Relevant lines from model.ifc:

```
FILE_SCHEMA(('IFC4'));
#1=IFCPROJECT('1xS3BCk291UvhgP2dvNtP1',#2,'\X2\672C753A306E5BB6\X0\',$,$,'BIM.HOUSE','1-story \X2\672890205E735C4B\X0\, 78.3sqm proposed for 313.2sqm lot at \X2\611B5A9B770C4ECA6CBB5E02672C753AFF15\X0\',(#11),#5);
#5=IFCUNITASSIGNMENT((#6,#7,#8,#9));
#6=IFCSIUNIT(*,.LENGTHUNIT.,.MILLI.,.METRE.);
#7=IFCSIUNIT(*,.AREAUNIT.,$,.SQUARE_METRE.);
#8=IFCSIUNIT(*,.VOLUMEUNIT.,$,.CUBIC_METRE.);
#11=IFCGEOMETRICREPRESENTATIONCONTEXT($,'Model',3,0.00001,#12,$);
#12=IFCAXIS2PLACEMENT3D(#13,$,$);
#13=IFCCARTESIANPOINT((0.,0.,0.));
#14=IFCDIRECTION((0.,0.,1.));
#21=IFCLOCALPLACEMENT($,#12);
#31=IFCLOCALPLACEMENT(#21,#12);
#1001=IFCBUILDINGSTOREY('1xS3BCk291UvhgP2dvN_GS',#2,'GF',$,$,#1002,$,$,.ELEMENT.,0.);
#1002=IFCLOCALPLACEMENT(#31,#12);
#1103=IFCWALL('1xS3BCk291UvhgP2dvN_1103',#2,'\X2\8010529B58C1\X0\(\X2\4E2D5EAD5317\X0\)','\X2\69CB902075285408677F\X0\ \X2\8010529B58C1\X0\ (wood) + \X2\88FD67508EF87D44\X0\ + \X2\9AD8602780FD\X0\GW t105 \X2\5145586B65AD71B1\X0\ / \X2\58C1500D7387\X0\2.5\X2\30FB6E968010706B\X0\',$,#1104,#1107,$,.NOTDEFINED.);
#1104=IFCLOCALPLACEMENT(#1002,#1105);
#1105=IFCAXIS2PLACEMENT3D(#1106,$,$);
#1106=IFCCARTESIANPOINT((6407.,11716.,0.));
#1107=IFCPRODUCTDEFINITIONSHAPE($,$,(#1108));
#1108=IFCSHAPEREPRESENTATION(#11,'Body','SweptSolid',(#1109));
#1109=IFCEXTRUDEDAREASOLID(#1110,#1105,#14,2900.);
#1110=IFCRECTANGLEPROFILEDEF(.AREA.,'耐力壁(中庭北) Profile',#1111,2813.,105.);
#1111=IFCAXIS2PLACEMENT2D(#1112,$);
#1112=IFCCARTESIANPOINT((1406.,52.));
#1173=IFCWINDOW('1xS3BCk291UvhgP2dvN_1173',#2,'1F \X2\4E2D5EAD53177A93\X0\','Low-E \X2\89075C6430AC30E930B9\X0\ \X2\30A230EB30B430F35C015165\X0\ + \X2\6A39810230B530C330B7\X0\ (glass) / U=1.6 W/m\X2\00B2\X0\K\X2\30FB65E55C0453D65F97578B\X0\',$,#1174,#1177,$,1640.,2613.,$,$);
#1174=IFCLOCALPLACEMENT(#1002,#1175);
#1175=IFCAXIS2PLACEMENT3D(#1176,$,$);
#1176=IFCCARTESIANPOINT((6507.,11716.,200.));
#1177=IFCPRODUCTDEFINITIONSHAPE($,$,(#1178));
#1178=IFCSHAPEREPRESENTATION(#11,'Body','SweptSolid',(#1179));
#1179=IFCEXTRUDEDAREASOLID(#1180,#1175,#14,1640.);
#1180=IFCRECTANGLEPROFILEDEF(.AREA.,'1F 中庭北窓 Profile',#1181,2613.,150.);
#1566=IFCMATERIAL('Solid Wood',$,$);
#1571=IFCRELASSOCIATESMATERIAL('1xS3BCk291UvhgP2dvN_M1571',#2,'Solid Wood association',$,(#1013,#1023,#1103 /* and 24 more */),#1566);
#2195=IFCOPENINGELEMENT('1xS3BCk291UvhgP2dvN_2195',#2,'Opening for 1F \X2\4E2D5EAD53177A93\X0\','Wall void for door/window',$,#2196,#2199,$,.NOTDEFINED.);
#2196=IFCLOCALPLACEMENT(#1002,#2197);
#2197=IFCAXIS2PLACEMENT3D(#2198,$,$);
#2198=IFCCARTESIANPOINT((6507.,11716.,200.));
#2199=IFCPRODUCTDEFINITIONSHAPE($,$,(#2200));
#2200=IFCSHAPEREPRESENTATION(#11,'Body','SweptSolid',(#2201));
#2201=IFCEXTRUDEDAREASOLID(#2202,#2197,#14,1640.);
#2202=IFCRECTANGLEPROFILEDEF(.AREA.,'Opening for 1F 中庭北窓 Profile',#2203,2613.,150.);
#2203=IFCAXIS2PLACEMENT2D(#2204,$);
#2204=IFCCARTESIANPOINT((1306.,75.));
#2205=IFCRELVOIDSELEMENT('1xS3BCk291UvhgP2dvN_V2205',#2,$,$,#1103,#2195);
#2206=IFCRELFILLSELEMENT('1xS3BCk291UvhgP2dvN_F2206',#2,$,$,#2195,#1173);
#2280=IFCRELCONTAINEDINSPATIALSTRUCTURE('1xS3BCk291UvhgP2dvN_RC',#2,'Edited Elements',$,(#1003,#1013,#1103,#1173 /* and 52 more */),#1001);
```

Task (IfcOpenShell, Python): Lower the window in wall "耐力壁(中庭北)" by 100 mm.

```python
import numpy as np
import ifcopenshell
import ifcopenshell.api.geometry
import ifcopenshell.util.placement
import ifcopenshell.util.unit

model = ifcopenshell.open("model.ifc")
unit_scale = ifcopenshell.util.unit.calculate_unit_scale(model)

window = model.by_guid("1xS3BCk291UvhgP2dvN_1173")
opening = window.FillsVoids[0].RelatingOpeningElement
dz = -0.1 / unit_scale

shift = np.array([0.0, 0.0, dz])
# The window is not placed relative to its opening, so move both.
for product in (opening, window):
    matrix = ifcopenshell.util.placement.get_local_placement(product.ObjectPlacement)
    matrix[:3, 3] += shift
    ifcopenshell.api.geometry.edit_object_placement(model, product=product, matrix=matrix, is_si=False)

print(f"moved by {dz * unit_scale:+.3f} m")

model.write("model-out.ifc")
```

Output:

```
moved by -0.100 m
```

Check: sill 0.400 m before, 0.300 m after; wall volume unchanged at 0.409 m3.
